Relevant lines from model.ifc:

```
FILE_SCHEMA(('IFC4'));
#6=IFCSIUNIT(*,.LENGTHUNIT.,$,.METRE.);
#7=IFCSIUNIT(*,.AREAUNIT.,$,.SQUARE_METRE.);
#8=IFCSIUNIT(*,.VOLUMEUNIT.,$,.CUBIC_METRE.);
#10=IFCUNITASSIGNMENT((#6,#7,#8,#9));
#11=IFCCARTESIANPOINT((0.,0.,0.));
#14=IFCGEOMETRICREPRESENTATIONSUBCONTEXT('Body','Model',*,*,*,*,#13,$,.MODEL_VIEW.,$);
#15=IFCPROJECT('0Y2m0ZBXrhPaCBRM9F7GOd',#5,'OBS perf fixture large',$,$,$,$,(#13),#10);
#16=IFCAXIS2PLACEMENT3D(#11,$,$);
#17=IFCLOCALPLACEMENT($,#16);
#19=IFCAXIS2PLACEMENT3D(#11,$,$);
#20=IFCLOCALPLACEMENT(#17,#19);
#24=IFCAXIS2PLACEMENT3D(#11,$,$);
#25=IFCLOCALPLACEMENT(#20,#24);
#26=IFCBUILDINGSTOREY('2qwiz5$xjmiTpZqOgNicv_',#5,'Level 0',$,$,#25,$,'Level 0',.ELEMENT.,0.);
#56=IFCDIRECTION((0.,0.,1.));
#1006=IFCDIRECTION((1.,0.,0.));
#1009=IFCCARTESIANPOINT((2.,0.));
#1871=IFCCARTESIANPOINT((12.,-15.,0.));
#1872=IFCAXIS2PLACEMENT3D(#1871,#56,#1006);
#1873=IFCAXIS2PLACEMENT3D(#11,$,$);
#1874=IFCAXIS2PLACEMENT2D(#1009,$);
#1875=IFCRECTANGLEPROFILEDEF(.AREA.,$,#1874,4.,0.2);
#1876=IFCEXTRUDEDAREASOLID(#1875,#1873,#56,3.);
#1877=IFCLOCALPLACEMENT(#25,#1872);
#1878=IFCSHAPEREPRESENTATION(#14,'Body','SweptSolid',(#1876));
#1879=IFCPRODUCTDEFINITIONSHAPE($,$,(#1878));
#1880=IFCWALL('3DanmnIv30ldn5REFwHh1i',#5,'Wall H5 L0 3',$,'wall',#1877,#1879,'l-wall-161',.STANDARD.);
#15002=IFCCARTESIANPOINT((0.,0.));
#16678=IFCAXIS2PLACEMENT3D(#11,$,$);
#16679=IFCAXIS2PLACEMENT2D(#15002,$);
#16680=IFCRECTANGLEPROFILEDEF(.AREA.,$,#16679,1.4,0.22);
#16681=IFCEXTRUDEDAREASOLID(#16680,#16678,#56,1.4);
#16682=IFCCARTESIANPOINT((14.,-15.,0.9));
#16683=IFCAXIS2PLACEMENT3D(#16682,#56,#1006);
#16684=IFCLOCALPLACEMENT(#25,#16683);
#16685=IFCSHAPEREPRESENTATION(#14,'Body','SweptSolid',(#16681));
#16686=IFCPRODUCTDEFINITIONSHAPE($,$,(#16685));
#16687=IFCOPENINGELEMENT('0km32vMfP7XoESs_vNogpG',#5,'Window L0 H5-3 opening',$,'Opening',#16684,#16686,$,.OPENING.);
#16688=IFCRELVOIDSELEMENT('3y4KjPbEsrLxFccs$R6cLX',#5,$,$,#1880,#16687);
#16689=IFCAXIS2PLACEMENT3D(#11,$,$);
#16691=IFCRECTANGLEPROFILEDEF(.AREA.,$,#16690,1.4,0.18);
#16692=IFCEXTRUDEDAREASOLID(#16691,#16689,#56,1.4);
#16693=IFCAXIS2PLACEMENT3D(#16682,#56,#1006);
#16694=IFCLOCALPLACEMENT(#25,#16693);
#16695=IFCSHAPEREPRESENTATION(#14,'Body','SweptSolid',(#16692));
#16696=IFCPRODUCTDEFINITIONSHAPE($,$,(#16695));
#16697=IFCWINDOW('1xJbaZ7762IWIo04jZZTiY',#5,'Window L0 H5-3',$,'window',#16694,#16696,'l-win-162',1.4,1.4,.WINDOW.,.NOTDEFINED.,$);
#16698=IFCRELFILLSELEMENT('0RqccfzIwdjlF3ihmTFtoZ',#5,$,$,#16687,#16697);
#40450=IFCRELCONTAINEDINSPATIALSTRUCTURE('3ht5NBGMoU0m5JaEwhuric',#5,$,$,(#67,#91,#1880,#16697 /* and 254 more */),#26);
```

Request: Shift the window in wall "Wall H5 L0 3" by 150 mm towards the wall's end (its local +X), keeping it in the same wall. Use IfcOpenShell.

```python
import ifcopenshell
import ifcopenshell.api.geometry
import ifcopenshell.util.placement
import ifcopenshell.util.unit

model = ifcopenshell.open("model.ifc")
unit_scale = ifcopenshell.util.unit.calculate_unit_scale(model)

window = model.by_id(16697)
opening = window.FillsVoids[0].RelatingOpeningElement
wall = opening.VoidsElements[0].RelatingBuildingElement

wall_matrix = ifcopenshell.util.placement.get_local_placement(wall.ObjectPlacement)
shift = wall_matrix[:3, 0] * 0.15 / unit_scale
before = ifcopenshell.util.placement.get_local_placement(window.ObjectPlacement)[:3, 3].copy()

# The window is not placed relative to its opening, so move both.
for product in (opening, window):
    matrix = ifcopenshell.util.placement.get_local_placement(product.ObjectPlacement)
    matrix[:3, 3] += shift
    ifcopenshell.api.geometry.edit_object_placement(model, product=product, matrix=matrix, is_si=False)

after = ifcopenshell.util.placement.get_local_placement(window.ObjectPlacement)[:3, 3]
print("window moved by", (after - before).round(3) + 0.0)

model.write("model_v2.ifc")
```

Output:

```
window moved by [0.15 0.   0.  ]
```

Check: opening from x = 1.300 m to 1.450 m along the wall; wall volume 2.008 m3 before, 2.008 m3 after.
